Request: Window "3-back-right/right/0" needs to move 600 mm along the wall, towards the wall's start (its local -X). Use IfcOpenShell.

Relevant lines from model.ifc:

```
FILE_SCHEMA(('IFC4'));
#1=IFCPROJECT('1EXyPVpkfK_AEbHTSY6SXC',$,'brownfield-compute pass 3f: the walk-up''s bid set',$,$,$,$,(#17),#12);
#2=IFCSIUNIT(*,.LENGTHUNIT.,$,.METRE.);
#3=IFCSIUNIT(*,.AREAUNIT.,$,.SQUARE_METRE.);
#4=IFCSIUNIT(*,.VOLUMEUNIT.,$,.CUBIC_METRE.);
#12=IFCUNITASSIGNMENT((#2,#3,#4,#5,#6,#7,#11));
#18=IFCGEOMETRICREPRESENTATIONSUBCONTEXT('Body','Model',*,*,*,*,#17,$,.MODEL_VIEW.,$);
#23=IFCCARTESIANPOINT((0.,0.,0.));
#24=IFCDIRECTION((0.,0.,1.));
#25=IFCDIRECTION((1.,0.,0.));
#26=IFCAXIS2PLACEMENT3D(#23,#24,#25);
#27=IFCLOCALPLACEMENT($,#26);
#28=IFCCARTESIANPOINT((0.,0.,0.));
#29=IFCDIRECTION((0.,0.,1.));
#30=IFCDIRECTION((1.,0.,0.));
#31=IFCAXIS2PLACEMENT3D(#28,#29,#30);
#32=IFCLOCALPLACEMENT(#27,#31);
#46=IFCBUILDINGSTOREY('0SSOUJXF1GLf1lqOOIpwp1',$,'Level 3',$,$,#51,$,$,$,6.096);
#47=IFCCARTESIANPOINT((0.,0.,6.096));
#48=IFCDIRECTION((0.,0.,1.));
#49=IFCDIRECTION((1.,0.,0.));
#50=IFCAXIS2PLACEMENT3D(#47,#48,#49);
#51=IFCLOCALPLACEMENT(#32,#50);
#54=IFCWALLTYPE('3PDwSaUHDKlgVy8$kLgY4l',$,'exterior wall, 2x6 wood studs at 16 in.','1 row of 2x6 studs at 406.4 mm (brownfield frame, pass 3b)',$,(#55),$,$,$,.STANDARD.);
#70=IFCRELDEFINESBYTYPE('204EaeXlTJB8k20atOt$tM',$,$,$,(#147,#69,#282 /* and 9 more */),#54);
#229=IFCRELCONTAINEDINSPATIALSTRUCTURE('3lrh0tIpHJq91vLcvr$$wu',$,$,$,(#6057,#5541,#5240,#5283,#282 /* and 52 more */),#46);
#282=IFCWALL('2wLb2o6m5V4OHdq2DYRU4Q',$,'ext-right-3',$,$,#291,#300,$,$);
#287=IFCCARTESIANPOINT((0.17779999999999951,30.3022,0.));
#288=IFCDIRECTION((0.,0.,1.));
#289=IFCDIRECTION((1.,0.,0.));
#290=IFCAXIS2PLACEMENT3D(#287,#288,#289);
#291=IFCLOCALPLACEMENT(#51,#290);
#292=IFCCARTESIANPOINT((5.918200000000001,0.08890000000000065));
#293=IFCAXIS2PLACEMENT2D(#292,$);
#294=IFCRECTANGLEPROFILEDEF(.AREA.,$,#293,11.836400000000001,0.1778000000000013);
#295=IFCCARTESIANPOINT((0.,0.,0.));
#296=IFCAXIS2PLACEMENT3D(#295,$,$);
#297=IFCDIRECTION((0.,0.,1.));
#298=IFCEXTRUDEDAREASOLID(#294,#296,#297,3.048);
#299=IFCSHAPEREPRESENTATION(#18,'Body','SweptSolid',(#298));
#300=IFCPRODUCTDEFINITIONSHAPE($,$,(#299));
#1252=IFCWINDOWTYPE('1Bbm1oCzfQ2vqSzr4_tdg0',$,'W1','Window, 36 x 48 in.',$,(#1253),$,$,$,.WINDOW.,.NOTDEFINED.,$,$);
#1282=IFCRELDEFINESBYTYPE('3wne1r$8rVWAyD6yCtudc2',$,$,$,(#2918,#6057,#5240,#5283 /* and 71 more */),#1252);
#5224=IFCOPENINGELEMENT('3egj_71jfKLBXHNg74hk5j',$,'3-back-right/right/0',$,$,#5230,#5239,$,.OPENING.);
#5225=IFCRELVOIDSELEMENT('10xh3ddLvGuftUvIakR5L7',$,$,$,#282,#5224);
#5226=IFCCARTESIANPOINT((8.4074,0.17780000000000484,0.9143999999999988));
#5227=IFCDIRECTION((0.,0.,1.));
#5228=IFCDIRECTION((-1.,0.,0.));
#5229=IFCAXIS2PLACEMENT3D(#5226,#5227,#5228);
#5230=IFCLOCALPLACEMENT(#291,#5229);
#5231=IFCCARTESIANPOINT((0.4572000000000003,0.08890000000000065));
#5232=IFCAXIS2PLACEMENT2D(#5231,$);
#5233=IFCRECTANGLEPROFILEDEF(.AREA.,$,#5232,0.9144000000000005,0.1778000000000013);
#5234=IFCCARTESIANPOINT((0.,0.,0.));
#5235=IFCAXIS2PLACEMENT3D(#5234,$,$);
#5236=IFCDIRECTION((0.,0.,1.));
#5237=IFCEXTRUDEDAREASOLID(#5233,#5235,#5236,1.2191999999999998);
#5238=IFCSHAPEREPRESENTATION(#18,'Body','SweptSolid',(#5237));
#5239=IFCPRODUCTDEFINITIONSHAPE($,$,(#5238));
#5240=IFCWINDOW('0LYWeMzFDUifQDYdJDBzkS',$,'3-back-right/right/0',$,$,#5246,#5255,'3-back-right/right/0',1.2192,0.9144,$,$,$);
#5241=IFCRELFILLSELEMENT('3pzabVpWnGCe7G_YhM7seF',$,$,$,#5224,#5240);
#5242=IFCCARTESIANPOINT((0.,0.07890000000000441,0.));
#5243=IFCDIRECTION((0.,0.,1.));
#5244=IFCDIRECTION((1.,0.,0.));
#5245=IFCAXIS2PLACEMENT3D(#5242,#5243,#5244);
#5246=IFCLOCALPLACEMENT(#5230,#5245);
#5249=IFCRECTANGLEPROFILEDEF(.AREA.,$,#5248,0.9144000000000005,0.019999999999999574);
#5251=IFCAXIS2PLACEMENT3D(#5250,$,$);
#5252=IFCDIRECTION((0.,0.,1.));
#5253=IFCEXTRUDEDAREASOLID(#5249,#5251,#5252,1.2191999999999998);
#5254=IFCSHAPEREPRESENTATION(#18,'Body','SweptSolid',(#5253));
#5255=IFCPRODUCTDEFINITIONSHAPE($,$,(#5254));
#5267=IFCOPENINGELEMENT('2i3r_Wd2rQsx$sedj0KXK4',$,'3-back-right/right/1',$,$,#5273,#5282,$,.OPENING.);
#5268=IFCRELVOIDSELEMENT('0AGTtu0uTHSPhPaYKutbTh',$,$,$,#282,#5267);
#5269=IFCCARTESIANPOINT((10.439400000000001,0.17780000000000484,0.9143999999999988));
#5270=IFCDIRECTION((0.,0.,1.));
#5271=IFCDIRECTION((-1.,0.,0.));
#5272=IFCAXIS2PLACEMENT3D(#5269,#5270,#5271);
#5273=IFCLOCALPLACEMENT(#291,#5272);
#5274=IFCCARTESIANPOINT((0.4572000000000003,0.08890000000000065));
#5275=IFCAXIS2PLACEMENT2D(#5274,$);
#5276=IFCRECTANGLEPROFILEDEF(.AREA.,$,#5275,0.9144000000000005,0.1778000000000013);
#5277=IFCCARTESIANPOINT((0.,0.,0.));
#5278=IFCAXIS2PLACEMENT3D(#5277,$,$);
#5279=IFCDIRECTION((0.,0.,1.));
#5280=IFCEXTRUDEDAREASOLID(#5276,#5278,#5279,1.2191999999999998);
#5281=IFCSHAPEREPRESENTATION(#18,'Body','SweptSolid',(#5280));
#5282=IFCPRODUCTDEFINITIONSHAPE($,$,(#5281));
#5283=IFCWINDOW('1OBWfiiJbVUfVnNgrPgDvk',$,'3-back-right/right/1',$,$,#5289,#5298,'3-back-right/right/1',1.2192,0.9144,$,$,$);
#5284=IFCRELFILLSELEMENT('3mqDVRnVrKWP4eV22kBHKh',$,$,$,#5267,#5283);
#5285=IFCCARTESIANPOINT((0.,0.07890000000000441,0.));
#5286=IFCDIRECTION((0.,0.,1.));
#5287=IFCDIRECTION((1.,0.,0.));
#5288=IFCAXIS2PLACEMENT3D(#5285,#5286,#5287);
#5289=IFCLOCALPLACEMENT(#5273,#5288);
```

```python
import ifcopenshell
import ifcopenshell.api.geometry
import ifcopenshell.util.placement

model = ifcopenshell.open("model.ifc")

window = model.by_id(5240)
opening = window.FillsVoids[0].RelatingOpeningElement
wall = opening.VoidsElements[0].RelatingBuildingElement

wall_matrix = ifcopenshell.util.placement.get_local_placement(wall.ObjectPlacement)
shift = wall_matrix[:3, 0] * -0.6
before = ifcopenshell.util.placement.get_local_placement(window.ObjectPlacement)[:3, 3].copy()

# The window is placed relative to its opening, so it follows when the opening moves.
matrix = ifcopenshell.util.placement.get_local_placement(opening.ObjectPlacement)
matrix[:3, 3] += shift
ifcopenshell.api.geometry.edit_object_placement(
    model, product=opening, matrix=matrix, is_si=False, should_transform_children=True
)

after = ifcopenshell.util.placement.get_local_placement(window.ObjectPlacement)[:3, 3]
print("window moved by", (after - before).round(3) + 0.0)

model.write("model_v2.ifc")
```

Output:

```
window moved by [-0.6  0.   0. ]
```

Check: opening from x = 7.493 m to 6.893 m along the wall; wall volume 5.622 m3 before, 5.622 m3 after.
